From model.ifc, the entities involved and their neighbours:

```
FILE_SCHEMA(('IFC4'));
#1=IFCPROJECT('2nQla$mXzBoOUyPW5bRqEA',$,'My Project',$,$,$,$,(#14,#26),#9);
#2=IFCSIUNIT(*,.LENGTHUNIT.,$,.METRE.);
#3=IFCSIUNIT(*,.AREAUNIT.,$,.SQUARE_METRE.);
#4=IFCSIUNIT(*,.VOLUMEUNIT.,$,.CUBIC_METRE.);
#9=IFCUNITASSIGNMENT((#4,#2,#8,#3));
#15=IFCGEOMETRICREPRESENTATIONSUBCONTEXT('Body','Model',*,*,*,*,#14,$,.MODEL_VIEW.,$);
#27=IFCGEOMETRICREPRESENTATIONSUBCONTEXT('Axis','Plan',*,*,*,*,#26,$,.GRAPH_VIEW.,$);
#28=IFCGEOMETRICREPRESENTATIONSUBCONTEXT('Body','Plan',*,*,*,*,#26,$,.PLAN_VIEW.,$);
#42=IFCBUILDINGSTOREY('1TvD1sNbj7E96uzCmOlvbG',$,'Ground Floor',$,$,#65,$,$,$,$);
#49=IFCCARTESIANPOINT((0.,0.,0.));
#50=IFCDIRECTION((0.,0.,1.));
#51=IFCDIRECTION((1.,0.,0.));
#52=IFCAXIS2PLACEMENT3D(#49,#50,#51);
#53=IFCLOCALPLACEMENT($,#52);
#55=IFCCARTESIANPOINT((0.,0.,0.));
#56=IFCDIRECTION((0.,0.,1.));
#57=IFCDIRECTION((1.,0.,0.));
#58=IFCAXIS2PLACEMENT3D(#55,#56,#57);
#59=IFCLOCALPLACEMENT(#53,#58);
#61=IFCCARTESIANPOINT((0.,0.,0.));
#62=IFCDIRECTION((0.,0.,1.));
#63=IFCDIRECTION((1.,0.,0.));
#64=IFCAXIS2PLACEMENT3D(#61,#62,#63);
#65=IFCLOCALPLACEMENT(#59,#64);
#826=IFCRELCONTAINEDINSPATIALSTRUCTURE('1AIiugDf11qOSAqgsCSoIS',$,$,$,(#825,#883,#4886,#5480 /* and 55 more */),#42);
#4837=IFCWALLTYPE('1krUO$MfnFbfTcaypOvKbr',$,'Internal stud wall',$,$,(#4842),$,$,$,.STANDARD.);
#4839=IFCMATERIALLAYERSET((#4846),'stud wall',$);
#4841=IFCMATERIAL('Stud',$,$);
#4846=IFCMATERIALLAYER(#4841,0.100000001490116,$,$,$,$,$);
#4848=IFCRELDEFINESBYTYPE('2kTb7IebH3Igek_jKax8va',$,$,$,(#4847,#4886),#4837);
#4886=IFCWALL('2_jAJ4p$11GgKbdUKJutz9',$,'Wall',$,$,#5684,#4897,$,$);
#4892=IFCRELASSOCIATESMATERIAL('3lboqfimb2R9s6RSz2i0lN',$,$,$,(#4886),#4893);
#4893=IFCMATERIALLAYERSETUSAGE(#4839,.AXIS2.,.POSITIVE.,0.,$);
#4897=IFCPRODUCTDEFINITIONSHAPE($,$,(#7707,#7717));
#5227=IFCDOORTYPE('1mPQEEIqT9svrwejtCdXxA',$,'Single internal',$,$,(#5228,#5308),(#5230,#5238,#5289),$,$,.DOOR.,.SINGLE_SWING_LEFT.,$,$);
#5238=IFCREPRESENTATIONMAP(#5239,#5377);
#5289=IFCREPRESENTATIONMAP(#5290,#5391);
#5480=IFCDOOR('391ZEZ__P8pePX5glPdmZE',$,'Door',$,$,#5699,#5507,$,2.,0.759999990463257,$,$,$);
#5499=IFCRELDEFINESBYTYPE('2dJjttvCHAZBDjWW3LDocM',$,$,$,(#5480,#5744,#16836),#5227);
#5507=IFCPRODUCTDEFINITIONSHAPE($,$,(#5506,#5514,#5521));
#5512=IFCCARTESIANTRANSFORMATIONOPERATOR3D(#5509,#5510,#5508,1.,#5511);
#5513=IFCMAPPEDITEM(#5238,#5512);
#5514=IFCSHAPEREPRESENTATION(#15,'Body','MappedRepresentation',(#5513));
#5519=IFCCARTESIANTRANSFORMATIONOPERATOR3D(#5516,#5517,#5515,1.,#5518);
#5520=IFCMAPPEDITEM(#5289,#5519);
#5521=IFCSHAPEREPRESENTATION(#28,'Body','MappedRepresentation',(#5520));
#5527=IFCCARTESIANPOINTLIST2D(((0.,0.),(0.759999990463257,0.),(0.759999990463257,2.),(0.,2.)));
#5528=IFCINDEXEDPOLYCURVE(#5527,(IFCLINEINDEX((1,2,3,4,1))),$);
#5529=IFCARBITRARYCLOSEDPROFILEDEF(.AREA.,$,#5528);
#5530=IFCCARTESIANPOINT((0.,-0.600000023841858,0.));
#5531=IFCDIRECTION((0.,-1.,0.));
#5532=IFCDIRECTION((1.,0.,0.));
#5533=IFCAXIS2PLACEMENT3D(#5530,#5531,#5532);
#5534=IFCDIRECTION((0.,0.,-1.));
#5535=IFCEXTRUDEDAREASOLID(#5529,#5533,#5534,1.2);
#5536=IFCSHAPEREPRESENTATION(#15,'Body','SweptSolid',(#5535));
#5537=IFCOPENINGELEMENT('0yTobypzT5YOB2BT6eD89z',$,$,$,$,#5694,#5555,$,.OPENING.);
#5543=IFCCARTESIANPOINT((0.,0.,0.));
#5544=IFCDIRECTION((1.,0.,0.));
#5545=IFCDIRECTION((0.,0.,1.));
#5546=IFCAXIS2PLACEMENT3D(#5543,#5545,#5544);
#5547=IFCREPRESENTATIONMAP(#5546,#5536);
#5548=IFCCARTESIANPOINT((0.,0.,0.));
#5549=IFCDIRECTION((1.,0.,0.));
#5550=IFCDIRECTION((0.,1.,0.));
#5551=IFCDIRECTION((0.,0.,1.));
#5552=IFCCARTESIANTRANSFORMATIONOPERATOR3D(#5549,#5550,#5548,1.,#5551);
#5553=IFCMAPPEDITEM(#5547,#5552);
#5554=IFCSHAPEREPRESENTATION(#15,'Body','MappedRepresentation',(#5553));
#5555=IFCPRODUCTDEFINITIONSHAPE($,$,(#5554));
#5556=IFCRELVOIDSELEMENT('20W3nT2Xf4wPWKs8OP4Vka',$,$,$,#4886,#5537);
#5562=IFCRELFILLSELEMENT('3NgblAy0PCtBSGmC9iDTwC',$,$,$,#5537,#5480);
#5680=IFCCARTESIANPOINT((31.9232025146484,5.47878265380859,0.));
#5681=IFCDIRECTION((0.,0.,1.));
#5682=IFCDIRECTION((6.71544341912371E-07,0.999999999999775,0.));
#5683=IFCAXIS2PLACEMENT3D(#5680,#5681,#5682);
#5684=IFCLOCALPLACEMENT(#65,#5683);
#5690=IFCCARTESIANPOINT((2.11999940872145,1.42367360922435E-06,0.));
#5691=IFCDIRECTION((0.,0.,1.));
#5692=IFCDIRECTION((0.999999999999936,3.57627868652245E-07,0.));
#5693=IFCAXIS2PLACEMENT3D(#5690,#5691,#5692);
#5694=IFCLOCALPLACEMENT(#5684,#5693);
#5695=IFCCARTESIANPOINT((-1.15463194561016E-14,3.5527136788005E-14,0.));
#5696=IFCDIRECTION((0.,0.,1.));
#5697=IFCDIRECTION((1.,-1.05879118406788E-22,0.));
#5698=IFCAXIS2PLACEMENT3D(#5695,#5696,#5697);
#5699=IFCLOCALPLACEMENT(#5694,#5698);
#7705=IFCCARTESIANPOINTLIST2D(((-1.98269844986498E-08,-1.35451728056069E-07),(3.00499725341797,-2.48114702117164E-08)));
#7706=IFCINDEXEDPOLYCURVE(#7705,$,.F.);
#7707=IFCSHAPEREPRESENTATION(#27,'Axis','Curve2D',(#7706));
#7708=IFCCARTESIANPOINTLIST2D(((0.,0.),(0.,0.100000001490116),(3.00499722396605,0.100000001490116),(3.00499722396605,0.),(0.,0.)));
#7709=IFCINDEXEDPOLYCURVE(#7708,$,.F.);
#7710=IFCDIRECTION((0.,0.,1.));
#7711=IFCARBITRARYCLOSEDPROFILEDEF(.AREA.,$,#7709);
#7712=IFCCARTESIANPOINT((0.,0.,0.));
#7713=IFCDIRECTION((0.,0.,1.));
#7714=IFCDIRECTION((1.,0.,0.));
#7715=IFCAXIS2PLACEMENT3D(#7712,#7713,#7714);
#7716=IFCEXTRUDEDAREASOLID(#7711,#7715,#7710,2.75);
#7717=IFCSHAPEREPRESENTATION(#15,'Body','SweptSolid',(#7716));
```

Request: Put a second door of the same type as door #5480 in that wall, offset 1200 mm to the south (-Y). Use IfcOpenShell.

```python
import ifcopenshell
import ifcopenshell.api.feature
import ifcopenshell.api.geometry
import ifcopenshell.api.root
import ifcopenshell.geom
import ifcopenshell.util.element
import ifcopenshell.util.placement
import ifcopenshell.util.shape
import ifcopenshell.util.unit

model = ifcopenshell.open("model.ifc")
unit_scale = ifcopenshell.util.unit.calculate_unit_scale(model)
settings = ifcopenshell.geom.settings()


def volume(element):
    """Net volume in cubic metres, openings subtracted."""
    shape = ifcopenshell.geom.create_shape(settings, element)
    return ifcopenshell.util.shape.get_volume(shape.geometry)


door = model.by_guid("391ZEZ__P8pePX5glPdmZE")
opening = door.FillsVoids[0].RelatingOpeningElement
wall = opening.VoidsElements[0].RelatingBuildingElement
before = volume(wall)
shift = ifcopenshell.util.placement.get_local_placement(wall.ObjectPlacement)[:3, 0] * -1.2 / unit_scale

# copy_class copies the void relationship, type, container and properties, but no geometry.
new_opening = ifcopenshell.api.root.copy_class(model, product=opening)
new_opening.Representation = ifcopenshell.util.element.copy_deep(
    model, opening.Representation, exclude=["IfcGeometricRepresentationContext", "IfcRepresentationMap"]
)
new_door = ifcopenshell.api.root.copy_class(model, product=door)
new_door.Representation = ifcopenshell.util.element.copy_deep(
    model, door.Representation, exclude=["IfcGeometricRepresentationContext", "IfcRepresentationMap"]
)
ifcopenshell.api.feature.add_filling(model, opening=new_opening, element=new_door)

for old, new in ((opening, new_opening), (door, new_door)):
    matrix = ifcopenshell.util.placement.get_local_placement(old.ObjectPlacement)
    matrix[:3, 3] += shift
    ifcopenshell.api.geometry.edit_object_placement(model, product=new, matrix=matrix, is_si=False)

after = volume(wall)

print(f"wall volume {before:.3f} -> {after:.3f} m3")

model.write("model_v2.ifc")
```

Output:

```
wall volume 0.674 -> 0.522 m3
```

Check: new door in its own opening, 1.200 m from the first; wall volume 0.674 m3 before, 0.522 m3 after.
